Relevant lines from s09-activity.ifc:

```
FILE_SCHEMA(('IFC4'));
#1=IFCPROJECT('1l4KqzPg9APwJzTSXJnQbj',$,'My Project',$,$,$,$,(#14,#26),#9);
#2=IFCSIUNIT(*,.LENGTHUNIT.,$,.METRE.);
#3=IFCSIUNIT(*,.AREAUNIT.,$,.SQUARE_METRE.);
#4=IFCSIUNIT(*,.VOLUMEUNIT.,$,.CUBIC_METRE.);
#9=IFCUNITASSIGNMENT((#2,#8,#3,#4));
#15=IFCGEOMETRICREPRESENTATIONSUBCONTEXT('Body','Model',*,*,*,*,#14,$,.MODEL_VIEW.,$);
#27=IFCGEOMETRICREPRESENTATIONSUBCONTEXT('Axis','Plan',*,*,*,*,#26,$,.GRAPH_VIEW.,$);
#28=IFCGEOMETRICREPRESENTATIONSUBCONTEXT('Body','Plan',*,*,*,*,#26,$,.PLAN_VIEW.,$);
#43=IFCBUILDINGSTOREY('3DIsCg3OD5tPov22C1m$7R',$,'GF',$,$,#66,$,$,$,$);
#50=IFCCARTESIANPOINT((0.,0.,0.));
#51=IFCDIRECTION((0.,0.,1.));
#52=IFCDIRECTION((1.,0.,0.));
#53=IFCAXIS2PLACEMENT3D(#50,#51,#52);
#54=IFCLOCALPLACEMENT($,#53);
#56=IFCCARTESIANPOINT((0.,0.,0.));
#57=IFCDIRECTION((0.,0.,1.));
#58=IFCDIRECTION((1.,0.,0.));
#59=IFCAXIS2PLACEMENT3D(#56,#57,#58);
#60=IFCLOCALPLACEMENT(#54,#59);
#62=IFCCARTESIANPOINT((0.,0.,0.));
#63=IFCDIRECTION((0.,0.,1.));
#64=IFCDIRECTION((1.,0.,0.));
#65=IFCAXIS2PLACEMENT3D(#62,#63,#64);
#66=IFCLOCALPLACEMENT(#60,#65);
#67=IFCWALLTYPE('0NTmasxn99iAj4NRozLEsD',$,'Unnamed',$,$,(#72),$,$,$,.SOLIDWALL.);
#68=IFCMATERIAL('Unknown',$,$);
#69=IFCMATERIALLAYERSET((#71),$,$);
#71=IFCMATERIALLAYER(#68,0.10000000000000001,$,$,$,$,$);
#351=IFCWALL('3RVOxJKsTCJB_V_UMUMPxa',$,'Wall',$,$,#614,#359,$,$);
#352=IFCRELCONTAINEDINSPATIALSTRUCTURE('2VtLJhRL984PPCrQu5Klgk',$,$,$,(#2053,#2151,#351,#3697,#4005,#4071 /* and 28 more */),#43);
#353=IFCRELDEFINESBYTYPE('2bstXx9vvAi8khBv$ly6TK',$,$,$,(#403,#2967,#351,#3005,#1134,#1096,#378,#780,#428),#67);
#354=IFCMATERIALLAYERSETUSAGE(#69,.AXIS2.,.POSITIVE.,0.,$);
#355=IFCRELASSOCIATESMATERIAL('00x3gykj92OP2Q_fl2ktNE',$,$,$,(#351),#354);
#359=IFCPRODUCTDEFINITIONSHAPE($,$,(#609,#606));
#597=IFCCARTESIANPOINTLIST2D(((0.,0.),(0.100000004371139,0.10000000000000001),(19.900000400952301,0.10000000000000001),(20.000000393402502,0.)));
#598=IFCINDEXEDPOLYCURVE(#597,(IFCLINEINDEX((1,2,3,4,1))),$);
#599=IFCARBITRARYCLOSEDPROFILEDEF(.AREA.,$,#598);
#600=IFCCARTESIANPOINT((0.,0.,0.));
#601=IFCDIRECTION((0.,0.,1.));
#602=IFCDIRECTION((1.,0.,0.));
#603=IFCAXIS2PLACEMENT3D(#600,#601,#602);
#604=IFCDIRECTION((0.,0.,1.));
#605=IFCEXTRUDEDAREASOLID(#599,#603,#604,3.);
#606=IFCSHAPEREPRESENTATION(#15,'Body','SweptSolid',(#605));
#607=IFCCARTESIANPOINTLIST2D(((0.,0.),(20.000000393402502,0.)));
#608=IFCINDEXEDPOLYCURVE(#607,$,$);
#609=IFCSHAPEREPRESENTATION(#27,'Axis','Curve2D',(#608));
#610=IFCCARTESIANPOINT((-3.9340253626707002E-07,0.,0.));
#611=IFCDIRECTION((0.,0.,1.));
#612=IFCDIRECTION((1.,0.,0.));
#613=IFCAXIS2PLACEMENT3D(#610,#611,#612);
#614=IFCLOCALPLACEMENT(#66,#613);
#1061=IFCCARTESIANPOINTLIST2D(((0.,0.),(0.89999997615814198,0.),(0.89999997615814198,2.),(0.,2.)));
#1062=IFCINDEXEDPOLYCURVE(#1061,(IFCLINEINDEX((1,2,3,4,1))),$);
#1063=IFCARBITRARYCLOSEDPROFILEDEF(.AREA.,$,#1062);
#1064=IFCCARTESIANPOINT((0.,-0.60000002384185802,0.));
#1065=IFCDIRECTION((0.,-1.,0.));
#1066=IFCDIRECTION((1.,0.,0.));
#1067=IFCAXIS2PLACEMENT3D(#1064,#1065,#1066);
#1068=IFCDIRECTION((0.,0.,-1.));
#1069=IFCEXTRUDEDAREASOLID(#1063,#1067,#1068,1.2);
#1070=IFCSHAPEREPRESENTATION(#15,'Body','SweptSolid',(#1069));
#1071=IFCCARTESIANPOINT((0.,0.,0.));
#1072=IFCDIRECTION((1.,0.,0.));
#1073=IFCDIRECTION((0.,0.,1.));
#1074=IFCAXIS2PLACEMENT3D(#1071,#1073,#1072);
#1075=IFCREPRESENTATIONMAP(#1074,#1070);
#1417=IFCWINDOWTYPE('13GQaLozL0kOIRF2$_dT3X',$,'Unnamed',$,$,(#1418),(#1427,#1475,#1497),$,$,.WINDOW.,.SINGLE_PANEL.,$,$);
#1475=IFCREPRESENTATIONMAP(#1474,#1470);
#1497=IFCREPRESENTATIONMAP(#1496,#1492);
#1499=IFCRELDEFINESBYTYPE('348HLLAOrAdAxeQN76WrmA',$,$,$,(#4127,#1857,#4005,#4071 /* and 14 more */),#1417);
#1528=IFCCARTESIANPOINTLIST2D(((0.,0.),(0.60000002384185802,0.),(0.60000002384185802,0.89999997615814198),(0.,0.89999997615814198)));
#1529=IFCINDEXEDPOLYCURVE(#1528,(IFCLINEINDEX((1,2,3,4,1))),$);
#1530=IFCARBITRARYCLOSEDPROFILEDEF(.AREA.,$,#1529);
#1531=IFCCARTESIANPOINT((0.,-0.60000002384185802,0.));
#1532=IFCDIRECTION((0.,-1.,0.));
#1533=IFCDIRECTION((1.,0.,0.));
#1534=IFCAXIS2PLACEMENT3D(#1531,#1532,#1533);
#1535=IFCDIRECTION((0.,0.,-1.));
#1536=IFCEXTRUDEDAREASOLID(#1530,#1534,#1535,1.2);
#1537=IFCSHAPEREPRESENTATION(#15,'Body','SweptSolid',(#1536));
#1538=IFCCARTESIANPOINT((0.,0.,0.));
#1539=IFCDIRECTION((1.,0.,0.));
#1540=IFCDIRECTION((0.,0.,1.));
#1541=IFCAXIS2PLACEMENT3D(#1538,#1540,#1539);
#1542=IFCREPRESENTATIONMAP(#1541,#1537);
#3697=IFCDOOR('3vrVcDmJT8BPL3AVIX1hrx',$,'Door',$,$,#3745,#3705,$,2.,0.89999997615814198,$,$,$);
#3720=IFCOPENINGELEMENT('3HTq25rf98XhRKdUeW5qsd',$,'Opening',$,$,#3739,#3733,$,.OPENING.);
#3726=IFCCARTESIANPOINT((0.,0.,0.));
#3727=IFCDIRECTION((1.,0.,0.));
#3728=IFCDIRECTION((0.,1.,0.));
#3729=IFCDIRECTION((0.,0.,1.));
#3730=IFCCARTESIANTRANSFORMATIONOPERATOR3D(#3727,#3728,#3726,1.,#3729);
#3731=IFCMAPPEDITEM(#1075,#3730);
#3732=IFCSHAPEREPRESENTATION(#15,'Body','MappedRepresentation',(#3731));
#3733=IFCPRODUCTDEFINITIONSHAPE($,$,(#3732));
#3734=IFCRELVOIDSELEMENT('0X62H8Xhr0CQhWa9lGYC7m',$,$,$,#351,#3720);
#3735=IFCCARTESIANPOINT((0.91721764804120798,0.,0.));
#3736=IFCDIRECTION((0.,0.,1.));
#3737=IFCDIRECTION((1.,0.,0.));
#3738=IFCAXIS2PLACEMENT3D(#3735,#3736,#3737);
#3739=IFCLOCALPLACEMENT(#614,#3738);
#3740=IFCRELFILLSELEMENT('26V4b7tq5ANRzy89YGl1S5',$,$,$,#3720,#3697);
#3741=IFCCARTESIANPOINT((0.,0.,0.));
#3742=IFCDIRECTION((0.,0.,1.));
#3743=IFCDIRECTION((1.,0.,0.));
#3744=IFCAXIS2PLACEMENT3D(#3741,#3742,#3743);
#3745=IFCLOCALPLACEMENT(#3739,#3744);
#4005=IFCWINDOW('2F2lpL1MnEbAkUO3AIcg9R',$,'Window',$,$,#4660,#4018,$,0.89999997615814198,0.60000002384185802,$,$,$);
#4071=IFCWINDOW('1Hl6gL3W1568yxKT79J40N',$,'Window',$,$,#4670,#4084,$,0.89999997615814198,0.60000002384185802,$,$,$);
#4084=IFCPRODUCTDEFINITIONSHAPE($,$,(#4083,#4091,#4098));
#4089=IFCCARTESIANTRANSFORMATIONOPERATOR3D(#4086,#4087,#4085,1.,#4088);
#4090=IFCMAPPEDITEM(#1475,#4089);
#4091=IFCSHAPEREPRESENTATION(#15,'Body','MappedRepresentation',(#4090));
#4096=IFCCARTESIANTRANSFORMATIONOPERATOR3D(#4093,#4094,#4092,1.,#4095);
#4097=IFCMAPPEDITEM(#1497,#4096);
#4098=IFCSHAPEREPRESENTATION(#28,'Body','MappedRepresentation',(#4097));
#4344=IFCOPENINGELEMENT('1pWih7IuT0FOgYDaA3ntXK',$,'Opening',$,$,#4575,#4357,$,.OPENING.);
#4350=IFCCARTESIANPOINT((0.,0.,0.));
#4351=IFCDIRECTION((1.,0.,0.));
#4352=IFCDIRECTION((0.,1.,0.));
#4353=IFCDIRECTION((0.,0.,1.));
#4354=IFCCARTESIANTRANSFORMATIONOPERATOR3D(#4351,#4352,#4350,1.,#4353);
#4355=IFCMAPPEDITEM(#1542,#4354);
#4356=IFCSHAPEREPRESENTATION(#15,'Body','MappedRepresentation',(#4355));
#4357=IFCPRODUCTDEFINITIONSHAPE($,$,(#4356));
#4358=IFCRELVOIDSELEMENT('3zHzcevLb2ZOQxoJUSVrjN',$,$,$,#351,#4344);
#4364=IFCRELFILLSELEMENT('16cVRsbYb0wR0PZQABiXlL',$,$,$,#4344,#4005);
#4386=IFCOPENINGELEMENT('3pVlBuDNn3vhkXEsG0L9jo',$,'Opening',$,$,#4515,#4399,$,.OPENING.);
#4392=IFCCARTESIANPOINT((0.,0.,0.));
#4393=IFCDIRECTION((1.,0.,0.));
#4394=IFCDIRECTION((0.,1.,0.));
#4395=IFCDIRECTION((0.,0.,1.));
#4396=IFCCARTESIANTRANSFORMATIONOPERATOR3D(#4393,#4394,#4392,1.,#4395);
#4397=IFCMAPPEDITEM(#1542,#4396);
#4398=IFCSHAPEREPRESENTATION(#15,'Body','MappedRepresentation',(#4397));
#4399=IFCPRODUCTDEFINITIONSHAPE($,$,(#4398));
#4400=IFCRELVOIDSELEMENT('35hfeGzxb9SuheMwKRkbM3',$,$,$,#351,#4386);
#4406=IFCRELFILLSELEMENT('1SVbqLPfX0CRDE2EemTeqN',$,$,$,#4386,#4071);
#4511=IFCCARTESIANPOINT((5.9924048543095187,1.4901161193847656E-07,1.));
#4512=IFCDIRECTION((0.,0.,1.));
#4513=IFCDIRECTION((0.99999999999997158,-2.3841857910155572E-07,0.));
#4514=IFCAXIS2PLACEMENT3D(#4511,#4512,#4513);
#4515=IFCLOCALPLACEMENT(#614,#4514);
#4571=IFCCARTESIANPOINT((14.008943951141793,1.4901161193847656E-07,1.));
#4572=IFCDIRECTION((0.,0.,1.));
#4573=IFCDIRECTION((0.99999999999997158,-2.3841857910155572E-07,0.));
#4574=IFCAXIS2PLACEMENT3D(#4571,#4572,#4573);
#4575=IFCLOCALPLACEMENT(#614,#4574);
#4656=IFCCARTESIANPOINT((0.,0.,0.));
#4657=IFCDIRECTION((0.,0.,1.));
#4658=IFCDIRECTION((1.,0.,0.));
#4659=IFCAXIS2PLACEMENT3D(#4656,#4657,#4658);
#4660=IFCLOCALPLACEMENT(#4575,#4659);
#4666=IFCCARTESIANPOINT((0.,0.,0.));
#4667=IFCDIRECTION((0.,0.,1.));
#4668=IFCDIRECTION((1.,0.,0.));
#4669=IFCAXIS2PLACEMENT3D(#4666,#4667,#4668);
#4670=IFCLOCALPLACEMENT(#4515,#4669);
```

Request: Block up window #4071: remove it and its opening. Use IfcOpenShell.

```python
import ifcopenshell
import ifcopenshell.api.feature
import ifcopenshell.api.root
import ifcopenshell.geom
import ifcopenshell.util.shape

model = ifcopenshell.open("s09-activity.ifc")
settings = ifcopenshell.geom.settings()


def volume(element):
    """Net volume in cubic metres, openings subtracted."""
    shape = ifcopenshell.geom.create_shape(settings, element)
    return ifcopenshell.util.shape.get_volume(shape.geometry)


window = model.by_id(4071)
opening = window.FillsVoids[0].RelatingOpeningElement
wall = opening.VoidsElements[0].RelatingBuildingElement
before = volume(wall)

ifcopenshell.api.root.remove_product(model, product=window)
ifcopenshell.api.feature.remove_feature(model, feature=opening)

after = volume(wall)

print(f"wall volume {before:.3f} -> {after:.3f} m3")

model.write("s09-activity_rev.ifc")
```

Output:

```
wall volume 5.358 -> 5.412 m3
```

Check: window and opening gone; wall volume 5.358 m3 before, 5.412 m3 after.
